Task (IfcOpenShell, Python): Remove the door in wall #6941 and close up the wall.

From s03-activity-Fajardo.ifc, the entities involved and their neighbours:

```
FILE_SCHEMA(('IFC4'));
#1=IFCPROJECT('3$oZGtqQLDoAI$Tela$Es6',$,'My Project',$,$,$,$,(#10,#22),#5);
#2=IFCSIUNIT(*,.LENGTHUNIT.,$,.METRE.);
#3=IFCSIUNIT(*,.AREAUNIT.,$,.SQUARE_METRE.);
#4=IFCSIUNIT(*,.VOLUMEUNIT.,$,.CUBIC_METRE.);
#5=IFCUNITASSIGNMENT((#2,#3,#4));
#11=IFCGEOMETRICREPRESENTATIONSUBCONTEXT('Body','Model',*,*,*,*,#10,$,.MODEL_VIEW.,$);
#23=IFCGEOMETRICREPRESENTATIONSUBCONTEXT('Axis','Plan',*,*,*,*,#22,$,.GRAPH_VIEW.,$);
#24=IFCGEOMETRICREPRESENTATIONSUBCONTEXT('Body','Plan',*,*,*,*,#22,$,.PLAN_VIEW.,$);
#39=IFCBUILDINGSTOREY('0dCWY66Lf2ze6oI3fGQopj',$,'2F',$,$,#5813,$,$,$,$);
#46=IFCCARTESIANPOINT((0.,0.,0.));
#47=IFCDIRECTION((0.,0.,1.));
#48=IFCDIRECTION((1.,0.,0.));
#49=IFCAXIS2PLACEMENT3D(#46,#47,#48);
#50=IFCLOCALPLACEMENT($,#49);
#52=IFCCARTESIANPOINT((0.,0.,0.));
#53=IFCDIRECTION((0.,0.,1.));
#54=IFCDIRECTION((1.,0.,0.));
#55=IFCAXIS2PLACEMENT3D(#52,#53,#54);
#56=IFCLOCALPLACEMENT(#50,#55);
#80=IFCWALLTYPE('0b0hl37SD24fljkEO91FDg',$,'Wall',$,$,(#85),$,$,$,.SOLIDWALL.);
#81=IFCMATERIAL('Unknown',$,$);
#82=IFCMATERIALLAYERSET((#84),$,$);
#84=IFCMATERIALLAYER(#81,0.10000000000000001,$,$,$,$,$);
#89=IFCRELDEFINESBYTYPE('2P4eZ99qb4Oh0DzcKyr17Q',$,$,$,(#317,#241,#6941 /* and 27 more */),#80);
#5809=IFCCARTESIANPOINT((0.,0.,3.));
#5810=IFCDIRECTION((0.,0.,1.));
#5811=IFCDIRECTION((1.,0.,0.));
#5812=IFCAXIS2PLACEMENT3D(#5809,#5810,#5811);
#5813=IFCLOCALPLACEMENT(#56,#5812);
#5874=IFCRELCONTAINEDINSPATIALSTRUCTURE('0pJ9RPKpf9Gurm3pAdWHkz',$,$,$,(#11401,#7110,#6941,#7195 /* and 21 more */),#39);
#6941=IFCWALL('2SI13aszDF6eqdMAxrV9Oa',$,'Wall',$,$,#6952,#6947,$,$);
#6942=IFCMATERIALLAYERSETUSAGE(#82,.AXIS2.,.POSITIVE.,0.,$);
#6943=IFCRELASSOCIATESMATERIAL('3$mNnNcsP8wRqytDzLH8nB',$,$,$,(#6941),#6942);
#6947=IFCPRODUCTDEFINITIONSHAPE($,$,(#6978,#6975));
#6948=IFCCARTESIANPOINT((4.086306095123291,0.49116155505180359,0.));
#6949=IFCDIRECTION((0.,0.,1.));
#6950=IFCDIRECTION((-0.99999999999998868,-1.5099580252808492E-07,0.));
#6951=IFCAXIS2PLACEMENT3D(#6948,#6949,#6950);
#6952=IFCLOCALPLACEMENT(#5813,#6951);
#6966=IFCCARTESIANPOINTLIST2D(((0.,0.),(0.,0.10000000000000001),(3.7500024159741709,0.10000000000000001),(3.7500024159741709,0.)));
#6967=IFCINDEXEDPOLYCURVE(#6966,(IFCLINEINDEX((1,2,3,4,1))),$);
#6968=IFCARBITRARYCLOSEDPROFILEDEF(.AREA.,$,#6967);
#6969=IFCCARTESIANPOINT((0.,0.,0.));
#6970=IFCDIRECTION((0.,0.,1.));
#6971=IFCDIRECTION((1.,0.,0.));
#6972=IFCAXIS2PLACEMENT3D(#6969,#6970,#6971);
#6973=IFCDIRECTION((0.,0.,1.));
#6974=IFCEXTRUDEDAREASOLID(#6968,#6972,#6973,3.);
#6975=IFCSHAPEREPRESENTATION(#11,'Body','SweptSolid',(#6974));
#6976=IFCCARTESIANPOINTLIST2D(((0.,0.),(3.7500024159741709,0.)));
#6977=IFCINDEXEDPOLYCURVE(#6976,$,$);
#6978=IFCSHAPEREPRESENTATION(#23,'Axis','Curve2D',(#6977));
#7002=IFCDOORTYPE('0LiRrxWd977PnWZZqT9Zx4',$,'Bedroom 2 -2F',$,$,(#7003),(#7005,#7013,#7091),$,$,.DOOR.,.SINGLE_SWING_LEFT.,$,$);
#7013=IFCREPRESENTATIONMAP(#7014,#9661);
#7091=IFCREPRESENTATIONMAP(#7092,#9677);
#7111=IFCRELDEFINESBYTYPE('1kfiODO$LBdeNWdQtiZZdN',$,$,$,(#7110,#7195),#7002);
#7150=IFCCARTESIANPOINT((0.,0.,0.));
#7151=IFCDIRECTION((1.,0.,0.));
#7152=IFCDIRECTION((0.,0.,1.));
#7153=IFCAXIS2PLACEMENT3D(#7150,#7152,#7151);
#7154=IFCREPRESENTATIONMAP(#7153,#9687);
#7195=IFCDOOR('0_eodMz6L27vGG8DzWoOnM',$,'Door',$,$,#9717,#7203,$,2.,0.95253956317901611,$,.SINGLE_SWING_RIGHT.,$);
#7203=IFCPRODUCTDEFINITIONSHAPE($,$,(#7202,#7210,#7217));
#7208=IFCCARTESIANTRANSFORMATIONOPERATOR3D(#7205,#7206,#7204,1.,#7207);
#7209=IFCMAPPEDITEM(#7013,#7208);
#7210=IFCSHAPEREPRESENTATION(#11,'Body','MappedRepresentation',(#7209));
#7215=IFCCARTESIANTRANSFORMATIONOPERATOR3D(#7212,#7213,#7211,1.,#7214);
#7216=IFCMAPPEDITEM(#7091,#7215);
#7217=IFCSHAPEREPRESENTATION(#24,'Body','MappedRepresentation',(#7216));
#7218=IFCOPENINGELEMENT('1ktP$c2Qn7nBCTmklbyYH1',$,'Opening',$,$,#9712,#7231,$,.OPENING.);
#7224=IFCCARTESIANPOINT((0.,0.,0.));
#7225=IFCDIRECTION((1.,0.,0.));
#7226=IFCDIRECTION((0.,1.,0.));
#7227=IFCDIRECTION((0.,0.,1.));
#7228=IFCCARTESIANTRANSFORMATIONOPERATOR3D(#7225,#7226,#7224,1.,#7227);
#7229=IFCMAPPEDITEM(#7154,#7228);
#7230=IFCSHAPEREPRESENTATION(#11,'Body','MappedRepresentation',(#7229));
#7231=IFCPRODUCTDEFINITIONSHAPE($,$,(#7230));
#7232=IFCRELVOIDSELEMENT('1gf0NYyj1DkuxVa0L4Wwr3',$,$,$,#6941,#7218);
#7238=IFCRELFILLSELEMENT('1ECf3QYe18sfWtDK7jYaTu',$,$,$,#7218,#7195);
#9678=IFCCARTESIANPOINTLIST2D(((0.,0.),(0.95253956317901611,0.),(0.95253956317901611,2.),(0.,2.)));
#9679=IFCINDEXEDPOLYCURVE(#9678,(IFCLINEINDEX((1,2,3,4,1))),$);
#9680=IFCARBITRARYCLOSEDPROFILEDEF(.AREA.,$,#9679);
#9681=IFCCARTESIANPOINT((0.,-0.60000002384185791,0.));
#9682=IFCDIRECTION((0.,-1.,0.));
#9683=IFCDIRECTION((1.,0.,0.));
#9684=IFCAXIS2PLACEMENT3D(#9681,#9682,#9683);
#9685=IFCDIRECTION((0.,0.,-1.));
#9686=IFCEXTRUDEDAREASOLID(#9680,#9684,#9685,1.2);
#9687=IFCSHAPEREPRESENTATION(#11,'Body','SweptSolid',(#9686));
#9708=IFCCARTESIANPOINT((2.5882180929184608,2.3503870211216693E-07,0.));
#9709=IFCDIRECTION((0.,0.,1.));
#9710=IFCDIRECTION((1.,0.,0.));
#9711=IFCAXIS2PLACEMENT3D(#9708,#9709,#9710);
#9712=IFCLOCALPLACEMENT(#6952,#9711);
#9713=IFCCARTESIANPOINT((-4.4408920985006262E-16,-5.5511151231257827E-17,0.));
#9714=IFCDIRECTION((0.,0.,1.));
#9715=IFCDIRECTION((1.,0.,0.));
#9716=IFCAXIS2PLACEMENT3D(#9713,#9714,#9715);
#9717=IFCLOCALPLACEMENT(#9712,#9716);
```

```python
import ifcopenshell
import ifcopenshell.api.feature
import ifcopenshell.api.root
import ifcopenshell.geom
import ifcopenshell.util.shape

model = ifcopenshell.open("s03-activity-Fajardo.ifc")
settings = ifcopenshell.geom.settings()


def volume(element):
    """Net volume in cubic metres, openings subtracted."""
    shape = ifcopenshell.geom.create_shape(settings, element)
    return ifcopenshell.util.shape.get_volume(shape.geometry)


door = model.by_guid("0_eodMz6L27vGG8DzWoOnM")
opening = door.FillsVoids[0].RelatingOpeningElement
wall = opening.VoidsElements[0].RelatingBuildingElement
before = volume(wall)

ifcopenshell.api.root.remove_product(model, product=door)
ifcopenshell.api.feature.remove_feature(model, feature=opening)

after = volume(wall)

print(f"wall volume {before:.3f} -> {after:.3f} m3")

model.write("s03-activity-Fajardo_rev.ifc")
```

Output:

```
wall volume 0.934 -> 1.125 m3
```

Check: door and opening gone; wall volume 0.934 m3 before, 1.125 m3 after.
